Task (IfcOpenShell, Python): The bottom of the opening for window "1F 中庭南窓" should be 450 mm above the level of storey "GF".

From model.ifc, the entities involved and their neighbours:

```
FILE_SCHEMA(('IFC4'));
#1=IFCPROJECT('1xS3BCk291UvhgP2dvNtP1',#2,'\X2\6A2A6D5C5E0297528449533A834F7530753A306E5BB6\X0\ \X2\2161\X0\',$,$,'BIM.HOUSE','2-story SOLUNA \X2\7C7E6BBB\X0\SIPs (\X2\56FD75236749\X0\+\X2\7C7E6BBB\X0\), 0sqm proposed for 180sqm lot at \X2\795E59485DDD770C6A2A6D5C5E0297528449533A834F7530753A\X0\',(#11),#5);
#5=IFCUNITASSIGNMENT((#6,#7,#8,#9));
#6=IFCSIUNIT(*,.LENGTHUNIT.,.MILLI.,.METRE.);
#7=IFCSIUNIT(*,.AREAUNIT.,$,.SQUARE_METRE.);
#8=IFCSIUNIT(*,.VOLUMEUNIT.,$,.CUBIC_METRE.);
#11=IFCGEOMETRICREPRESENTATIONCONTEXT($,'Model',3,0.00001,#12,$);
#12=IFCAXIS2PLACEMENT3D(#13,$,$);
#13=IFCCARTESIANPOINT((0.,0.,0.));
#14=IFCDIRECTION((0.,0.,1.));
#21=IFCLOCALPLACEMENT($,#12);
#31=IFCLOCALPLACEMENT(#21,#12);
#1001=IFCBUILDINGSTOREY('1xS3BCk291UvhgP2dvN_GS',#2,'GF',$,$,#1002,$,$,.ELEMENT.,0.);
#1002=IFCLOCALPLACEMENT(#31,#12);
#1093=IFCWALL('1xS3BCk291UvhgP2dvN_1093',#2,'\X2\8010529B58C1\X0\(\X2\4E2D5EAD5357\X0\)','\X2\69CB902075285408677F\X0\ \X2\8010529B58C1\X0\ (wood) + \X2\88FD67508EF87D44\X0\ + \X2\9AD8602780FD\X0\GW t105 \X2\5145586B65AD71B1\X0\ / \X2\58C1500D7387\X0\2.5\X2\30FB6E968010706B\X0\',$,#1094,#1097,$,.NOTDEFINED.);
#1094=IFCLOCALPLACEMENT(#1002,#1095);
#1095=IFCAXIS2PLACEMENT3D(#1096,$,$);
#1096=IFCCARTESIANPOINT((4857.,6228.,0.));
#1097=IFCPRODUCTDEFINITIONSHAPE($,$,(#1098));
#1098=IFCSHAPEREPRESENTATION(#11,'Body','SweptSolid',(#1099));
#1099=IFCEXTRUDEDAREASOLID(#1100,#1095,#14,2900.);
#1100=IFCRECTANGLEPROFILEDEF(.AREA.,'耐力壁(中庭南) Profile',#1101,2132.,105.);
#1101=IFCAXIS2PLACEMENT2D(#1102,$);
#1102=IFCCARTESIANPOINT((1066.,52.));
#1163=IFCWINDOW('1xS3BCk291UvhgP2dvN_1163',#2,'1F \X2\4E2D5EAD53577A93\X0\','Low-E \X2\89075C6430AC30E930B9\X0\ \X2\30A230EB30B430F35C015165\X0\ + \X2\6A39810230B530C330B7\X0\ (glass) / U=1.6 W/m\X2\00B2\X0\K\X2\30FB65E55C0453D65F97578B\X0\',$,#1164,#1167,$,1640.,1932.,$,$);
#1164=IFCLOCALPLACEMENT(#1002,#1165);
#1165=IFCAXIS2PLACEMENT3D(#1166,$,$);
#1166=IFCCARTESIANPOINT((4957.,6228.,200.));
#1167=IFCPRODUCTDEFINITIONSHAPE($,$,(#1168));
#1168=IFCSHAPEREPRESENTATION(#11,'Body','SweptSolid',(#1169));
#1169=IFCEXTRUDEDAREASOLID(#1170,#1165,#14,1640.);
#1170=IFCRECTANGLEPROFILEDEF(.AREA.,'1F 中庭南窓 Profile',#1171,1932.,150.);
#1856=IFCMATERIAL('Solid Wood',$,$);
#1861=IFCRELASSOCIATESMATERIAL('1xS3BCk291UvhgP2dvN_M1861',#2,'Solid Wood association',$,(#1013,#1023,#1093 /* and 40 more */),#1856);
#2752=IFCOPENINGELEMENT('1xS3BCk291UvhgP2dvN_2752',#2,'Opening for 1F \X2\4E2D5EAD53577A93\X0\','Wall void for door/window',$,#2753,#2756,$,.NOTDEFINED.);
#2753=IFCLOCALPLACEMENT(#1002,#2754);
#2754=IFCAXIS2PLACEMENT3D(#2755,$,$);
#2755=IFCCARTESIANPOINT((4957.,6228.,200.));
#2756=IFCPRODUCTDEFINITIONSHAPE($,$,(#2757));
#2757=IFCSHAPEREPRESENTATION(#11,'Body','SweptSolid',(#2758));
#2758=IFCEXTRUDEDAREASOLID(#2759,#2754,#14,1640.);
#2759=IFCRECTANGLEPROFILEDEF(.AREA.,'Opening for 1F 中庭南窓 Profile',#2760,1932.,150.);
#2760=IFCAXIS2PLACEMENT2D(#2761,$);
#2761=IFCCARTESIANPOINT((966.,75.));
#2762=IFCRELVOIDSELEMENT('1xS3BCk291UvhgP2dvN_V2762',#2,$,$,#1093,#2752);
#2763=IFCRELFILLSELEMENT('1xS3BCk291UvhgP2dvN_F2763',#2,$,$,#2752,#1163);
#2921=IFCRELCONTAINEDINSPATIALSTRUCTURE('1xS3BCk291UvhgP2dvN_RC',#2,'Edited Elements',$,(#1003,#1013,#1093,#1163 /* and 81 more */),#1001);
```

```python
import numpy as np
import ifcopenshell
import ifcopenshell.api.geometry
import ifcopenshell.geom
import ifcopenshell.util.element
import ifcopenshell.util.placement
import ifcopenshell.util.shape
import ifcopenshell.util.unit

model = ifcopenshell.open("model.ifc")
unit_scale = ifcopenshell.util.unit.calculate_unit_scale(model)

window = model.by_guid("1xS3BCk291UvhgP2dvN_1163")
opening = window.FillsVoids[0].RelatingOpeningElement
storey = ifcopenshell.util.element.get_container(window, ifc_class="IfcBuildingStorey")
level = ifcopenshell.util.placement.get_local_placement(storey.ObjectPlacement)[2, 3]

# The opening's origin need not be at the sill, so measure its lowest point.
shape = ifcopenshell.geom.create_shape(ifcopenshell.geom.settings(), opening)
bottom = ifcopenshell.util.shape.get_shape_bottom_elevation(shape, shape.geometry) / unit_scale
dz = level + 0.45 / unit_scale - bottom

shift = np.array([0.0, 0.0, dz])
# The window is not placed relative to its opening, so move both.
for product in (opening, window):
    matrix = ifcopenshell.util.placement.get_local_placement(product.ObjectPlacement)
    matrix[:3, 3] += shift
    ifcopenshell.api.geometry.edit_object_placement(model, product=product, matrix=matrix, is_si=False)

print(f"moved by {dz * unit_scale:+.3f} m")

model.write("model_rev.ifc")
```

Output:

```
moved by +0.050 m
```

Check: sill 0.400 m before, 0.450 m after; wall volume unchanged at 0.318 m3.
